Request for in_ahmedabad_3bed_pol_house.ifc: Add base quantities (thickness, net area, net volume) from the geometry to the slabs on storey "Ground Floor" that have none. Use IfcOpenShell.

First a look at what the model holds.

```python
import ifcopenshell
import ifcopenshell.util.element
import ifcopenshell.util.unit

model = ifcopenshell.open("in_ahmedabad_3bed_pol_house.ifc")
print(model.schema)
for unit_type in ("LENGTHUNIT", "AREAUNIT", "VOLUMEUNIT"):
    print(unit_type, ifcopenshell.util.unit.calculate_unit_scale(model, unit_type))
storey = next(s for s in model.by_type("IfcBuildingStorey") if s.Name == "Ground Floor")
slabs = [e for e in ifcopenshell.util.element.get_decomposition(storey) if e.is_a("IfcSlab")]
for e in sorted(slabs, key=lambda e: e.id()):
    print(e.id(), e.is_a(), e.Name, list(ifcopenshell.util.element.get_psets(e, qtos_only=True)), sep=" | ")
```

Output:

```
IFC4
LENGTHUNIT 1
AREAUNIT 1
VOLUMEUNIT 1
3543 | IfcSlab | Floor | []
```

```python
import ifcopenshell
import ifcopenshell.api.pset
import ifcopenshell.geom
import ifcopenshell.util.element
import ifcopenshell.util.shape
import ifcopenshell.util.unit

model = ifcopenshell.open("in_ahmedabad_3bed_pol_house.ifc")
unit_scale = ifcopenshell.util.unit.calculate_unit_scale(model)
area_scale = ifcopenshell.util.unit.calculate_unit_scale(model, "AREAUNIT")
volume_scale = ifcopenshell.util.unit.calculate_unit_scale(model, "VOLUMEUNIT")
settings = ifcopenshell.geom.settings()

storey = next(s for s in model.by_type("IfcBuildingStorey") if s.Name == "Ground Floor")
slabs = [e for e in ifcopenshell.util.element.get_decomposition(storey) if e.is_a("IfcSlab")]

for e in sorted(slabs, key=lambda e: e.id()):
    if ifcopenshell.util.element.get_psets(e, qtos_only=True, should_inherit=False):
        continue
    # Geometry comes back in metres, in the element's own axes.
    shape = ifcopenshell.geom.create_shape(settings, e)
    values = {
        "Width": ifcopenshell.util.shape.get_z(shape.geometry) / unit_scale,
        "NetArea": ifcopenshell.util.shape.get_footprint_area(shape.geometry) / area_scale,
        "NetVolume": ifcopenshell.util.shape.get_volume(shape.geometry) / volume_scale,
    }
    qto = ifcopenshell.api.pset.add_qto(model, product=e, name="Qto_SlabBaseQuantities")
    ifcopenshell.api.pset.edit_qto(model, qto=qto, properties=values)
    print(e.id(), {k: round(v, 3) for k, v in values.items()})

model.write("in_ahmedabad_3bed_pol_house_v2.ifc")
```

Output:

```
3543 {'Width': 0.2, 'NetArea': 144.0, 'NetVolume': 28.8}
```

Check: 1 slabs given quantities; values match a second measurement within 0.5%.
